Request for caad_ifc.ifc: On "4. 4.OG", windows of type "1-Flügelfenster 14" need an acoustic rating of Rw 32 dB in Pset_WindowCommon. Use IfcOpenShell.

First a look at what the model holds.

```python
import ifcopenshell
import ifcopenshell.util.element

model = ifcopenshell.open("caad_ifc.ifc")
print(model.schema)
storey = next(s for s in model.by_type("IfcBuildingStorey") if s.Name == "4. 4.OG")
windows = [e for e in ifcopenshell.util.element.get_decomposition(storey) if e.is_a("IfcWindow")]
seen = {}
for e in windows:
    element_type = ifcopenshell.util.element.get_type(e)
    key = (element_type.Name if element_type != e and element_type else None, ifcopenshell.util.element.get_pset(e, "Pset_WindowCommon", "AcousticRating"))
    seen[key] = seen.get(key, 0) + 1
for (name, value), count in sorted(seen.items(), key=str):
    print(count, "x", name, "|", value)
```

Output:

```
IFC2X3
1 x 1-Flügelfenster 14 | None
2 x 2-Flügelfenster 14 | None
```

```python
import ifcopenshell
import ifcopenshell.api.pset
import ifcopenshell.util.element

model = ifcopenshell.open("caad_ifc.ifc")

storey = next(s for s in model.by_type("IfcBuildingStorey") if s.Name == "4. 4.OG")
windows = [e for e in ifcopenshell.util.element.get_decomposition(storey) if e.is_a("IfcWindow")]

count = 0
for e in windows:
    element_type = ifcopenshell.util.element.get_type(e)
    if element_type in (None, e) or element_type.Name != "1-Flügelfenster 14":
        continue
    # add_pset returns the element's existing set when there is one.
    pset = ifcopenshell.api.pset.add_pset(model, product=e, name="Pset_WindowCommon")
    ifcopenshell.api.pset.edit_pset(model, pset=pset, properties={"AcousticRating": "Rw 32 dB"})
    count += 1

print(count, "windows updated")

model.write("caad_ifc_updated.ifc")
```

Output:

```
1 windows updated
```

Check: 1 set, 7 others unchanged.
